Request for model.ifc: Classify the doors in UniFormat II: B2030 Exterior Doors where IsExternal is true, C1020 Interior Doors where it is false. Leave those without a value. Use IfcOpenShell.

First a look at what the model holds.

```python
import ifcopenshell
import ifcopenshell.util.element

model = ifcopenshell.open("model.ifc")
print(model.schema)
print("classifications:", [c.Name for c in model.by_type("IfcClassification")])
values = [ifcopenshell.util.element.get_pset(e, "Pset_DoorCommon", "IsExternal") for e in model.by_type("IfcDoor")]
for value in (True, False, None):
    print("IsExternal", value, values.count(value))
```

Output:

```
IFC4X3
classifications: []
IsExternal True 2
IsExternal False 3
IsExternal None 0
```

```python
import ifcopenshell
import ifcopenshell.api.classification
import ifcopenshell.util.element

model = ifcopenshell.open("model.ifc")

system = ifcopenshell.api.classification.add_classification(model, classification="UniFormat II")

doors = model.by_type("IfcDoor")
external = {e: ifcopenshell.util.element.get_pset(e, "Pset_DoorCommon", "IsExternal") for e in doors}
for flag, code, name in ((True, "B2030", "Exterior Doors"), (False, "C1020", "Interior Doors")):
    products = [e for e in doors if external[e] is flag]
    ifcopenshell.api.classification.add_reference(
        model, products=products, classification=system, identification=code, name=name
    )
    print(code, len(products))

model.write("model_v2.ifc")
```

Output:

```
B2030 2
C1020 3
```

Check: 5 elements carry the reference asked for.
